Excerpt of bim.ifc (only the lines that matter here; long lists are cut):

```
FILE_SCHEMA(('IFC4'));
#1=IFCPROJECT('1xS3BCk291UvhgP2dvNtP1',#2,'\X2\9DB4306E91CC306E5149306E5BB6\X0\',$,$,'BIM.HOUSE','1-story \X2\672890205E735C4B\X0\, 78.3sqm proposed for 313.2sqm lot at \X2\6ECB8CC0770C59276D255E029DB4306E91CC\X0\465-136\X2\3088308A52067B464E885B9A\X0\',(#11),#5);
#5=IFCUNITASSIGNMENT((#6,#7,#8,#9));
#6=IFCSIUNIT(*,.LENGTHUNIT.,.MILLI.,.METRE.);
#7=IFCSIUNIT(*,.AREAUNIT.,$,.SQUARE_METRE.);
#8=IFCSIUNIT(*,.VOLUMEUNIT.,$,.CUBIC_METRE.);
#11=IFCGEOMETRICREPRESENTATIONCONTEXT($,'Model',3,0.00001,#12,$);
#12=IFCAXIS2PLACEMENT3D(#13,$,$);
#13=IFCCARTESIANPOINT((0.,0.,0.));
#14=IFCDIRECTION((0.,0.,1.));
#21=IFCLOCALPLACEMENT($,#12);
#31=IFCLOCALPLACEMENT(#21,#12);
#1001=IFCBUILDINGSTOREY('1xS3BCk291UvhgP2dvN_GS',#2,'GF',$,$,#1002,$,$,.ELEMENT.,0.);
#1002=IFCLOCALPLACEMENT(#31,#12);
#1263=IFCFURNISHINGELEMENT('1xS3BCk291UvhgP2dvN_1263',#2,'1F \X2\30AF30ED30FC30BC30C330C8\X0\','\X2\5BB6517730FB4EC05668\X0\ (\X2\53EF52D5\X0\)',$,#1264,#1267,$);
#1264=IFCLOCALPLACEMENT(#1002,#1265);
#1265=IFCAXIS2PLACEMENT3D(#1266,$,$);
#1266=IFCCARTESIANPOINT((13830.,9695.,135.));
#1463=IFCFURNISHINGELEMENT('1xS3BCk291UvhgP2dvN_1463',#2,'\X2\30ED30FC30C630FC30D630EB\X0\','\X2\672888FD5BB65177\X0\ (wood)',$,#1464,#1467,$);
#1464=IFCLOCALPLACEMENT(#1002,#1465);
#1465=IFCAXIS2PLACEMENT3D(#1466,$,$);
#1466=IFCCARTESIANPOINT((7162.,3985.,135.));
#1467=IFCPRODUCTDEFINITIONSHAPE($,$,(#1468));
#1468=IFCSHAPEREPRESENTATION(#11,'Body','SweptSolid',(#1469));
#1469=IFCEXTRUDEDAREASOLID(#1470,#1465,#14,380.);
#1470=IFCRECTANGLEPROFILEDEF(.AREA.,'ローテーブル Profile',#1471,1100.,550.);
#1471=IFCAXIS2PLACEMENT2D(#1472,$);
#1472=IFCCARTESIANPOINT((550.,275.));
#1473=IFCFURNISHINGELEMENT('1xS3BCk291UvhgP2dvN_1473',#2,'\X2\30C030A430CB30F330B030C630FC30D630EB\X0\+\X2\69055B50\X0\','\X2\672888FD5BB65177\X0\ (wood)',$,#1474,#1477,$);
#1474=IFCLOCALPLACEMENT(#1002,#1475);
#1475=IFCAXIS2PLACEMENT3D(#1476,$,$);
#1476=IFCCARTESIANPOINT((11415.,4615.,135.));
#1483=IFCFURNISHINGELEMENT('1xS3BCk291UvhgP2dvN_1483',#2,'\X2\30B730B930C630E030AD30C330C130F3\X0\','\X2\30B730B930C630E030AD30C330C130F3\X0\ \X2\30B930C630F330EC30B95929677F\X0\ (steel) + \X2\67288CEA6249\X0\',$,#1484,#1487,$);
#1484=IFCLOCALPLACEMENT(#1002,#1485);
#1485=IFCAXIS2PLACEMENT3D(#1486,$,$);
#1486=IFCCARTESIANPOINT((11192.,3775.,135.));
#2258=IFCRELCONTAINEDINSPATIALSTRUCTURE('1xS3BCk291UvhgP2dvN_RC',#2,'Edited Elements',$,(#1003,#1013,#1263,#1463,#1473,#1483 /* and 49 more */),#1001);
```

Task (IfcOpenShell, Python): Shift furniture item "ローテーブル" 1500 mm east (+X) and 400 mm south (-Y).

```python
import ifcopenshell
import ifcopenshell.api.geometry
import ifcopenshell.util.placement
import ifcopenshell.util.unit

model = ifcopenshell.open("bim.ifc")
unit_scale = ifcopenshell.util.unit.calculate_unit_scale(model)

item = model.by_guid("1xS3BCk291UvhgP2dvN_1463")
matrix = ifcopenshell.util.placement.get_local_placement(item.ObjectPlacement)
matrix[0, 3] += 1.5 / unit_scale
matrix[1, 3] -= 0.4 / unit_scale
ifcopenshell.api.geometry.edit_object_placement(model, product=item, matrix=matrix, is_si=False)

print(ifcopenshell.util.placement.get_local_placement(item.ObjectPlacement).round(3) + 0.0)

model.write("bim_v2.ifc")
```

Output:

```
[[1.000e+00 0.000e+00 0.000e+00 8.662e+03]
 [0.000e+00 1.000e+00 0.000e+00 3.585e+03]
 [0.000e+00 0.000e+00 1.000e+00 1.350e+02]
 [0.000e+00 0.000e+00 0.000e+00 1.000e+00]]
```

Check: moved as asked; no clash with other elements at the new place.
